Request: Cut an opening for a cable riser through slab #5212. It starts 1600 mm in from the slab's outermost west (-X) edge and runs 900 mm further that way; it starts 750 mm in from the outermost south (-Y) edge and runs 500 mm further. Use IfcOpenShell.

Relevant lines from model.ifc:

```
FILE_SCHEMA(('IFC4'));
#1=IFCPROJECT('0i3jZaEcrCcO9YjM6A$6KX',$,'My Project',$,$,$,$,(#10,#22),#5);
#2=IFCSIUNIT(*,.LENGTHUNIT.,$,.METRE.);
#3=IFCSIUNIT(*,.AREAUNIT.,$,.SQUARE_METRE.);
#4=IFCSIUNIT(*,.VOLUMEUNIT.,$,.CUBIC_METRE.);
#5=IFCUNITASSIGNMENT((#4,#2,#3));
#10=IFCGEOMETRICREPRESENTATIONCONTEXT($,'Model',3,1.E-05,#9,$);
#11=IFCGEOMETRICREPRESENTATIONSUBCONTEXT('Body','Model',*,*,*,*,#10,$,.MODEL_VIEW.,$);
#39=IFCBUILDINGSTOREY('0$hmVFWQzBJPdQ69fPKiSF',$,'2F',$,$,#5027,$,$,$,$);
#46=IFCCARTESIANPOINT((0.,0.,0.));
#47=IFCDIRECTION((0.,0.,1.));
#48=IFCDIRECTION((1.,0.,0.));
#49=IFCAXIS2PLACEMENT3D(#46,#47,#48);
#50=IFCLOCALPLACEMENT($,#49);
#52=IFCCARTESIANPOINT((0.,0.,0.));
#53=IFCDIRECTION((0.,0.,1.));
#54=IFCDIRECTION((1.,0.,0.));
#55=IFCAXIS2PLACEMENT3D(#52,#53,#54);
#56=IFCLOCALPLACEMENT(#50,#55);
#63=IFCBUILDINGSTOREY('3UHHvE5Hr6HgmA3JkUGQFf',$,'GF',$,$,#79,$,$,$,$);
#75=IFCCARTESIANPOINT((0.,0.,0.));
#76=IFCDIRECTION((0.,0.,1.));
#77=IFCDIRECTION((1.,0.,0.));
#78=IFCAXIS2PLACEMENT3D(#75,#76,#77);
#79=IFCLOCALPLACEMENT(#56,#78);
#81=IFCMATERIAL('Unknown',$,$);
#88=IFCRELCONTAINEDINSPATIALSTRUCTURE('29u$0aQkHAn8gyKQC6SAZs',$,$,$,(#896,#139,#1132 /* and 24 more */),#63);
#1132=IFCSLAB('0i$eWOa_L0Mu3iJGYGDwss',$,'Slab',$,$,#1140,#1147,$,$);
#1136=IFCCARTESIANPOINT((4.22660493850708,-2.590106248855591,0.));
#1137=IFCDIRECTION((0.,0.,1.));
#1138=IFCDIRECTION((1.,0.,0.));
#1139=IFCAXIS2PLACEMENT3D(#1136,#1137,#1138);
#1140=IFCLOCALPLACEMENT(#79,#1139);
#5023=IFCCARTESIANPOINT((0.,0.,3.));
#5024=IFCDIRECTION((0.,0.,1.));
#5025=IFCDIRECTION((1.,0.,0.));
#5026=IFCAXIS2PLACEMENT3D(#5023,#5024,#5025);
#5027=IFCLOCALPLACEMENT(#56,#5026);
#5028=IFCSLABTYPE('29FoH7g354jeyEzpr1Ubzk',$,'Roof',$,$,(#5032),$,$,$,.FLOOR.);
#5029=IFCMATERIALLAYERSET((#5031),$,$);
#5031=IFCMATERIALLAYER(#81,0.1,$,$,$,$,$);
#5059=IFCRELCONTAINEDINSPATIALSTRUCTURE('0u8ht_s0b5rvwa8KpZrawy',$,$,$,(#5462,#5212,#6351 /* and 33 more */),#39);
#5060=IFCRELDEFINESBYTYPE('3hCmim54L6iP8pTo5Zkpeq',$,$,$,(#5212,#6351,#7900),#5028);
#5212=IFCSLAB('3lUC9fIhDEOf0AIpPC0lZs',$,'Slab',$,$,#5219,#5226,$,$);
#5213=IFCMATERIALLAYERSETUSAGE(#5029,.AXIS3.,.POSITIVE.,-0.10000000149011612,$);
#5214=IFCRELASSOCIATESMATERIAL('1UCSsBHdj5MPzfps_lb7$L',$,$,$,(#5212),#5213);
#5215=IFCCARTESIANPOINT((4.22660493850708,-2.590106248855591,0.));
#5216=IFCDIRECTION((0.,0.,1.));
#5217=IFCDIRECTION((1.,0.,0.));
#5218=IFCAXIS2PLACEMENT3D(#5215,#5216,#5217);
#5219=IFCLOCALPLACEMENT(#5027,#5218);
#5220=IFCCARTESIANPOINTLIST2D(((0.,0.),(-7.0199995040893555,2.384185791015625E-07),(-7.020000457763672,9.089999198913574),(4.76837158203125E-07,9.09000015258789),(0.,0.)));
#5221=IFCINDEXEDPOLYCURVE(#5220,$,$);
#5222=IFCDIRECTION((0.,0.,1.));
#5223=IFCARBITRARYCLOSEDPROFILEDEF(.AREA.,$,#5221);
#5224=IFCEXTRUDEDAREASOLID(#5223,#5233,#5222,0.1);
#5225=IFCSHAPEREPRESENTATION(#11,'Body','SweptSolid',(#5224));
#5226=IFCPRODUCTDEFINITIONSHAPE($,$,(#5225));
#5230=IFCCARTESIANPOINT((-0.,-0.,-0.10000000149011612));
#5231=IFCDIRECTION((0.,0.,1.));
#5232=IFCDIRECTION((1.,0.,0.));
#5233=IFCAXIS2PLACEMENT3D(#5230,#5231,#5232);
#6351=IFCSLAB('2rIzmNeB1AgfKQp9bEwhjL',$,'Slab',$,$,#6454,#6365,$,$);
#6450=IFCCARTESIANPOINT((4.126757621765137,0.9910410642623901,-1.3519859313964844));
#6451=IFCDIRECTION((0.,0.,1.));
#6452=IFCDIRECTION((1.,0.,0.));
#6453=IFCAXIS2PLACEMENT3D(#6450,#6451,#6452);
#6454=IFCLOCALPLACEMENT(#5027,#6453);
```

```python
import numpy as np
import ifcopenshell
import ifcopenshell.api.feature
import ifcopenshell.api.geometry
import ifcopenshell.api.root
import ifcopenshell.geom
import ifcopenshell.util.placement
import ifcopenshell.util.representation
import ifcopenshell.util.shape
import ifcopenshell.util.unit

model = ifcopenshell.open("model.ifc")
unit_scale = ifcopenshell.util.unit.calculate_unit_scale(model)
settings = ifcopenshell.geom.settings()


def volume(element):
    """Net volume in cubic metres, openings subtracted."""
    shape = ifcopenshell.geom.create_shape(settings, element)
    return ifcopenshell.util.shape.get_volume(shape.geometry)


slab = model.by_guid("3lUC9fIhDEOf0AIpPC0lZs")
before = volume(slab)

# Extent in the slab's own axes, in metres. The edges named are its -X and -Y sides.
slab_shape = ifcopenshell.geom.create_shape(settings, slab)
vertices = ifcopenshell.util.shape.get_vertices(slab_shape.geometry)
x_min, y_min, bottom = vertices.min(axis=0)
top = vertices[:, 2].max()

opening = ifcopenshell.api.root.create_entity(model, ifc_class="IfcOpeningElement", name="Cable riser opening", predefined_type="OPENING")
context = ifcopenshell.util.representation.get_context(model, "Model", "Body", "MODEL_VIEW")
width, depth = 0.9, 0.5
outline = [(0.0, 0.0), (width, 0.0), (width, depth), (0.0, depth), (0.0, 0.0)]
# Overshoot both faces by 50 mm so the cut is clean.
shape = ifcopenshell.api.geometry.add_slab_representation(
    model, context=context, depth=top - bottom + 0.1, polyline=outline
)
ifcopenshell.api.geometry.assign_representation(model, product=opening, representation=shape)

matrix = ifcopenshell.util.placement.get_local_placement(slab.ObjectPlacement)
matrix[:, 3] = matrix @ np.append(np.array([x_min + 1.6, y_min + 0.75, bottom - 0.05]) / unit_scale, 1.0)
ifcopenshell.api.geometry.edit_object_placement(model, product=opening, matrix=matrix, is_si=False)
ifcopenshell.api.feature.add_feature(model, feature=opening, element=slab)

after = volume(slab)

print(f"slab volume {before:.3f} -> {after:.3f} m3")

model.write("model_edited.ifc")
```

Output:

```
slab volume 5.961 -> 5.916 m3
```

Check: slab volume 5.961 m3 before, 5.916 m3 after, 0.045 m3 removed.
